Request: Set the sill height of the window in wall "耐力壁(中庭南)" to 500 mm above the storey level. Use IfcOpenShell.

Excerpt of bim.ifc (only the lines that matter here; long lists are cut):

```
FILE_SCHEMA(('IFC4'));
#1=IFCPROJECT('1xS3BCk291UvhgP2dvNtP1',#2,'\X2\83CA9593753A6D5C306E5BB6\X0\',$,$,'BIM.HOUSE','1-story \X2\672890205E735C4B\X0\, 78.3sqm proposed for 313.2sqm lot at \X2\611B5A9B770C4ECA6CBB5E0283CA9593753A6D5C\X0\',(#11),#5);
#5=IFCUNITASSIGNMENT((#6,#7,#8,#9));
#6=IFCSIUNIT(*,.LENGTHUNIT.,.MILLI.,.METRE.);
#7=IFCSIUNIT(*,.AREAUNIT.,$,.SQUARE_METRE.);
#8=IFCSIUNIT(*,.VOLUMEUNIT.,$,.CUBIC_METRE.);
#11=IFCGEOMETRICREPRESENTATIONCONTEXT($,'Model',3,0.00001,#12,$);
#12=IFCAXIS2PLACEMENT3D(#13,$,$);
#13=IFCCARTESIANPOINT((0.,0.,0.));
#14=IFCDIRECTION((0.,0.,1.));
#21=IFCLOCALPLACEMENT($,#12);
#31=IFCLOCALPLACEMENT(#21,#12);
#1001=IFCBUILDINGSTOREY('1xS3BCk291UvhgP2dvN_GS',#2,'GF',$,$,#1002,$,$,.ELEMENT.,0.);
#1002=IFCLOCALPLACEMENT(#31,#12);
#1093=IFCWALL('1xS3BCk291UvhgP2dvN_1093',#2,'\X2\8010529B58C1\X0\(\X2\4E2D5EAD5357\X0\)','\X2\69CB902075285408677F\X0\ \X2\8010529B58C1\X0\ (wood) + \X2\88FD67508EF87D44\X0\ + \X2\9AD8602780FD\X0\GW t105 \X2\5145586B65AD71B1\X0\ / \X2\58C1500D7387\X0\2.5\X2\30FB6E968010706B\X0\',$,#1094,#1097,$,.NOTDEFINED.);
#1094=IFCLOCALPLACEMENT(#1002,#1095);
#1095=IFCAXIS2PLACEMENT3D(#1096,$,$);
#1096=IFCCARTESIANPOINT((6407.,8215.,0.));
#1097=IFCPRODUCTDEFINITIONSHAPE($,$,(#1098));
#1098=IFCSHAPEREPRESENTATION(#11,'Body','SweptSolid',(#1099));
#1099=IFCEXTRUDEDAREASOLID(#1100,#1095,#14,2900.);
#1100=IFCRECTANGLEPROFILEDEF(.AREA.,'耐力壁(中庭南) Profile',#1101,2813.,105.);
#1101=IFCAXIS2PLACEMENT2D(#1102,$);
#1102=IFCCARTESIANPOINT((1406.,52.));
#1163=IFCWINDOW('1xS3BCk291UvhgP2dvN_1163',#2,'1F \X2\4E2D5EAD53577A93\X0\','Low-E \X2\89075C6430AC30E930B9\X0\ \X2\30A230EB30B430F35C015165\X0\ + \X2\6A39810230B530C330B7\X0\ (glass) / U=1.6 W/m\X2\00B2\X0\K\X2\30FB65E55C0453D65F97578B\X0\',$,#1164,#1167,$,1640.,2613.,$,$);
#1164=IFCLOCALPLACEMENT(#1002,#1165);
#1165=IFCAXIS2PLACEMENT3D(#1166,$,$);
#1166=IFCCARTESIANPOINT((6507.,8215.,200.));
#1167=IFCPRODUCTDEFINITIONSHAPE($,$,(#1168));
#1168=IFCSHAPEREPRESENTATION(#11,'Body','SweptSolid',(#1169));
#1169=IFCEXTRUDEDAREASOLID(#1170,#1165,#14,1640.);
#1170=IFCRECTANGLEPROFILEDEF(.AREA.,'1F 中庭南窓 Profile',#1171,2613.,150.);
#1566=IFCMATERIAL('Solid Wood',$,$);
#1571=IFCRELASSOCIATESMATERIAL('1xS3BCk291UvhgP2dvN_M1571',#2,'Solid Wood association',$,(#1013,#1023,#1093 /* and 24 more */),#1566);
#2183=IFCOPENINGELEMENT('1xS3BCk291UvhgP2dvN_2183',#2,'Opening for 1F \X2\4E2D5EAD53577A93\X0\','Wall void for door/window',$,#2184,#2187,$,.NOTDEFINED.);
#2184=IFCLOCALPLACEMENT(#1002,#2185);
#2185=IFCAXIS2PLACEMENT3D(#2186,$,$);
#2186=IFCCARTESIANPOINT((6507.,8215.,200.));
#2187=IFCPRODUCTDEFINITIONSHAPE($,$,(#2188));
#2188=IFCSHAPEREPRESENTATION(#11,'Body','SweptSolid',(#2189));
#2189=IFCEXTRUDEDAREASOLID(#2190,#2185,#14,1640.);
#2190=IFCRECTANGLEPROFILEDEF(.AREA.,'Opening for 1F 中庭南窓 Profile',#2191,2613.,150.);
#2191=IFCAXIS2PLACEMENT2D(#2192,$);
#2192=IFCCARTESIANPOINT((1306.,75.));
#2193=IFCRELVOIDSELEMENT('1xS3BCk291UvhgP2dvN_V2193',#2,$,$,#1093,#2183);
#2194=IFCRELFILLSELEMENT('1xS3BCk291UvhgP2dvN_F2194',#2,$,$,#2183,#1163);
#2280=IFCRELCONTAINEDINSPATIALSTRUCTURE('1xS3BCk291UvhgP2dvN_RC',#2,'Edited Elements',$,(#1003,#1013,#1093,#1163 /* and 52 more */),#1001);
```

```python
import numpy as np
import ifcopenshell
import ifcopenshell.api.geometry
import ifcopenshell.geom
import ifcopenshell.util.element
import ifcopenshell.util.placement
import ifcopenshell.util.shape
import ifcopenshell.util.unit

model = ifcopenshell.open("bim.ifc")
unit_scale = ifcopenshell.util.unit.calculate_unit_scale(model)

window = model.by_guid("1xS3BCk291UvhgP2dvN_1163")
opening = window.FillsVoids[0].RelatingOpeningElement
storey = ifcopenshell.util.element.get_container(window, ifc_class="IfcBuildingStorey")
level = ifcopenshell.util.placement.get_local_placement(storey.ObjectPlacement)[2, 3]

# The opening's origin need not be at the sill, so measure its lowest point.
shape = ifcopenshell.geom.create_shape(ifcopenshell.geom.settings(), opening)
bottom = ifcopenshell.util.shape.get_shape_bottom_elevation(shape, shape.geometry) / unit_scale
dz = level + 0.5 / unit_scale - bottom

shift = np.array([0.0, 0.0, dz])
# The window is not placed relative to its opening, so move both.
for product in (opening, window):
    matrix = ifcopenshell.util.placement.get_local_placement(product.ObjectPlacement)
    matrix[:3, 3] += shift
    ifcopenshell.api.geometry.edit_object_placement(model, product=product, matrix=matrix, is_si=False)

print(f"moved by {dz * unit_scale:+.3f} m")

model.write("bim_v2.ifc")
```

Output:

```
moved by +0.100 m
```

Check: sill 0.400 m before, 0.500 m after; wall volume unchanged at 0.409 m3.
